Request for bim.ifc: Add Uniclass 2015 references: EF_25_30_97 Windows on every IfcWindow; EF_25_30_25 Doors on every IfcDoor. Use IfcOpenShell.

First a look at what the model holds.

```python
import ifcopenshell

model = ifcopenshell.open("bim.ifc")
print(model.schema)
print("classifications:", [c.Name for c in model.by_type("IfcClassification")])
for ifc_class in ("IfcDoor", "IfcRoof", "IfcStair", "IfcWall", "IfcWindow"):
    print(ifc_class, len(model.by_type(ifc_class)))
```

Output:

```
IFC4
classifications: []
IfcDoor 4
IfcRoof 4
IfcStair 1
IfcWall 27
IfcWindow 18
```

```python
import ifcopenshell
import ifcopenshell.api.classification

model = ifcopenshell.open("bim.ifc")

system = ifcopenshell.api.classification.add_classification(model, classification="Uniclass 2015")

codes = {
    "IfcWindow": ("EF_25_30_97", "Windows"),
    "IfcDoor": ("EF_25_30_25", "Doors"),
}
for ifc_class, (code, name) in codes.items():
    products = model.by_type(ifc_class)
    ifcopenshell.api.classification.add_reference(
        model, products=products, classification=system, identification=code, name=name
    )
    print(code, len(products))

model.write("bim-out.ifc")
```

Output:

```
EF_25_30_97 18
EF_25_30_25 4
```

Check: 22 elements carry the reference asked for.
